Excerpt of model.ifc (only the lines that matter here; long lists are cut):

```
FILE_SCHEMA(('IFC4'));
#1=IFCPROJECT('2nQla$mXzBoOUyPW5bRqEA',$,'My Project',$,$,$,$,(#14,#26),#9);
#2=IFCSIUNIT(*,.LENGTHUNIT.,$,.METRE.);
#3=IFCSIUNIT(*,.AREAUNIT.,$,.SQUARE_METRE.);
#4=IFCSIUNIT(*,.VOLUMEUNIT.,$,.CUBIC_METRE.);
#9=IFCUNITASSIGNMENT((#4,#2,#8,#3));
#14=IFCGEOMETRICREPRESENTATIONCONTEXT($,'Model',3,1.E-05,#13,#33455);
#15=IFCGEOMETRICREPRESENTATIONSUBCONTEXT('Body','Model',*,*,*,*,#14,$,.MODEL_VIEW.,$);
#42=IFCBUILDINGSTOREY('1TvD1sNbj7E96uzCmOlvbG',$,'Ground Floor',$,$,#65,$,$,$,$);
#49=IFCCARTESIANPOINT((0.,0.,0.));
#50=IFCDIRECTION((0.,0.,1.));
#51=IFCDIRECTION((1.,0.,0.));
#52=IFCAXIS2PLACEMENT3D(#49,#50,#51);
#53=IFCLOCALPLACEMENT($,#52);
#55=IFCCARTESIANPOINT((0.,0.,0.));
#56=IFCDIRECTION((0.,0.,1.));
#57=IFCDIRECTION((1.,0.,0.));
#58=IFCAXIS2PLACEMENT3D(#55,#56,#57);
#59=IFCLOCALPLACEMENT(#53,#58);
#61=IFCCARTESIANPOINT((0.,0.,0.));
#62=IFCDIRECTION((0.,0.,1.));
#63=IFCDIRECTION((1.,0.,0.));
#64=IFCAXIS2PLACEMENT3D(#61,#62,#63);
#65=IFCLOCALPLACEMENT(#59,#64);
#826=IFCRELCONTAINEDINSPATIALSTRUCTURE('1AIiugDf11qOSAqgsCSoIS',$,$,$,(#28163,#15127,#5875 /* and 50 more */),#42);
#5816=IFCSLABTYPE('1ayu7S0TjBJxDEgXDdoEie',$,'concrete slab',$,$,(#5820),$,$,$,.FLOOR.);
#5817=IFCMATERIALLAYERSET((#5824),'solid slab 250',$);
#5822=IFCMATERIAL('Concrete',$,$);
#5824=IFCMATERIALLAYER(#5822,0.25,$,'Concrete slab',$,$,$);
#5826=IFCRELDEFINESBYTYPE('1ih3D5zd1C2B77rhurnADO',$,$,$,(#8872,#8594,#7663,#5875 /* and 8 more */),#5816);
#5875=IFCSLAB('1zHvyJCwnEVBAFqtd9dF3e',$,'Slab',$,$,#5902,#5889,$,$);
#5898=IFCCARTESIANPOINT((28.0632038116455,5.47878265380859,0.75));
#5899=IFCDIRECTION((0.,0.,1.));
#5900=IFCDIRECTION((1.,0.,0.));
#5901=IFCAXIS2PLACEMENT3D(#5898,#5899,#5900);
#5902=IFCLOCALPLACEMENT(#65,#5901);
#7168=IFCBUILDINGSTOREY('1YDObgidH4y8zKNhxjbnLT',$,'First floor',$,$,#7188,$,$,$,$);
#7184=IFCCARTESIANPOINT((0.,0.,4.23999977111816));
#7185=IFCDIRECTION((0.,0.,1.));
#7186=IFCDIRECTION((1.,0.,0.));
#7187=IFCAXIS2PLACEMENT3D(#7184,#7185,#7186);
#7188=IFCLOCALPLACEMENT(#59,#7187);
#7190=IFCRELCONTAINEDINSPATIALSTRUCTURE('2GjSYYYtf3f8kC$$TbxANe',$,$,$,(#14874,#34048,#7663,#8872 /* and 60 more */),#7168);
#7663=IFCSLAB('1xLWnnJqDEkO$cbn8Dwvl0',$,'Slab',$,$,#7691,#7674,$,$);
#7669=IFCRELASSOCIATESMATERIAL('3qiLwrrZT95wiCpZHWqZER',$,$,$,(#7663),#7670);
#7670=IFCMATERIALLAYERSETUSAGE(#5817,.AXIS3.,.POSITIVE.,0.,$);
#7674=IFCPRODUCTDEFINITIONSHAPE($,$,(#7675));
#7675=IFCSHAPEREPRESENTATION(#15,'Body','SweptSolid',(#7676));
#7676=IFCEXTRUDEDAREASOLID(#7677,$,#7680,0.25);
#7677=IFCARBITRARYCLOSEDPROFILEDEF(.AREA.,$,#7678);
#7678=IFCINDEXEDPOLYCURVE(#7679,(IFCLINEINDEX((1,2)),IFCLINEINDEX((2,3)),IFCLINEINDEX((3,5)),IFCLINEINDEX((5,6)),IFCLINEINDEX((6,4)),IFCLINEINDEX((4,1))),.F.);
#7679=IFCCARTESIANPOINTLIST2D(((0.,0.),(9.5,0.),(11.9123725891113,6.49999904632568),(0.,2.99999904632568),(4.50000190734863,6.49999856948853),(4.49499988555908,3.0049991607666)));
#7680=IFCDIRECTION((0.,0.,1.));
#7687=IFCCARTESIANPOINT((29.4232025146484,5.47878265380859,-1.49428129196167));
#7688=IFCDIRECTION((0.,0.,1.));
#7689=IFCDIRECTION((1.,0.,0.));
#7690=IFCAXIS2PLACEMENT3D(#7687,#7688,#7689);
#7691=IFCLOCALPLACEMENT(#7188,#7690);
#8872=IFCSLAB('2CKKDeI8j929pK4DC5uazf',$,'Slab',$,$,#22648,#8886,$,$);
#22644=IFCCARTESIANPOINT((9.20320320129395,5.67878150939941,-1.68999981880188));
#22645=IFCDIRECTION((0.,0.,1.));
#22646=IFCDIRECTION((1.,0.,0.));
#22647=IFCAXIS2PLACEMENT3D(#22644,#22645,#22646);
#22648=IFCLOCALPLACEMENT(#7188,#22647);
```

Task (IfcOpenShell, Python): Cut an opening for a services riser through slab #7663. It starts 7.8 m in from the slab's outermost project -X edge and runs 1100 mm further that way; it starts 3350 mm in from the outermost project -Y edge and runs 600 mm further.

```python
import numpy as np
import ifcopenshell
import ifcopenshell.api.feature
import ifcopenshell.api.geometry
import ifcopenshell.api.root
import ifcopenshell.geom
import ifcopenshell.util.placement
import ifcopenshell.util.representation
import ifcopenshell.util.shape
import ifcopenshell.util.unit

model = ifcopenshell.open("model.ifc")
unit_scale = ifcopenshell.util.unit.calculate_unit_scale(model)
settings = ifcopenshell.geom.settings()


def volume(element):
    """Net volume in cubic metres, openings subtracted."""
    shape = ifcopenshell.geom.create_shape(settings, element)
    return ifcopenshell.util.shape.get_volume(shape.geometry)


slab = model.by_id(7663)
before = volume(slab)

# Extent in the slab's own axes, in metres. The edges named are its -X and -Y sides.
slab_shape = ifcopenshell.geom.create_shape(settings, slab)
vertices = ifcopenshell.util.shape.get_vertices(slab_shape.geometry)
x_min, y_min, bottom = vertices.min(axis=0)
top = vertices[:, 2].max()

opening = ifcopenshell.api.root.create_entity(model, ifc_class="IfcOpeningElement", name="Services riser opening", predefined_type="OPENING")
context = ifcopenshell.util.representation.get_context(model, "Model", "Body", "MODEL_VIEW")
width, depth = 1.1, 0.6
outline = [(0.0, 0.0), (width, 0.0), (width, depth), (0.0, depth), (0.0, 0.0)]
# Overshoot both faces by 50 mm so the cut is clean.
shape = ifcopenshell.api.geometry.add_slab_representation(
    model, context=context, depth=top - bottom + 0.1, polyline=outline
)
ifcopenshell.api.geometry.assign_representation(model, product=opening, representation=shape)

matrix = ifcopenshell.util.placement.get_local_placement(slab.ObjectPlacement)
matrix[:, 3] = matrix @ np.append(np.array([x_min + 7.8, y_min + 3.35, bottom - 0.05]) / unit_scale, 1.0)
ifcopenshell.api.geometry.edit_object_placement(model, product=opening, matrix=matrix, is_si=False)
ifcopenshell.api.feature.add_feature(model, feature=opening, element=slab)

after = volume(slab)

print(f"slab volume {before:.3f} -> {after:.3f} m3")

model.write("model_rev.ifc")
```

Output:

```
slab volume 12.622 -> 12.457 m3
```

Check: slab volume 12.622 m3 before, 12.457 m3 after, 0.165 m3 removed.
